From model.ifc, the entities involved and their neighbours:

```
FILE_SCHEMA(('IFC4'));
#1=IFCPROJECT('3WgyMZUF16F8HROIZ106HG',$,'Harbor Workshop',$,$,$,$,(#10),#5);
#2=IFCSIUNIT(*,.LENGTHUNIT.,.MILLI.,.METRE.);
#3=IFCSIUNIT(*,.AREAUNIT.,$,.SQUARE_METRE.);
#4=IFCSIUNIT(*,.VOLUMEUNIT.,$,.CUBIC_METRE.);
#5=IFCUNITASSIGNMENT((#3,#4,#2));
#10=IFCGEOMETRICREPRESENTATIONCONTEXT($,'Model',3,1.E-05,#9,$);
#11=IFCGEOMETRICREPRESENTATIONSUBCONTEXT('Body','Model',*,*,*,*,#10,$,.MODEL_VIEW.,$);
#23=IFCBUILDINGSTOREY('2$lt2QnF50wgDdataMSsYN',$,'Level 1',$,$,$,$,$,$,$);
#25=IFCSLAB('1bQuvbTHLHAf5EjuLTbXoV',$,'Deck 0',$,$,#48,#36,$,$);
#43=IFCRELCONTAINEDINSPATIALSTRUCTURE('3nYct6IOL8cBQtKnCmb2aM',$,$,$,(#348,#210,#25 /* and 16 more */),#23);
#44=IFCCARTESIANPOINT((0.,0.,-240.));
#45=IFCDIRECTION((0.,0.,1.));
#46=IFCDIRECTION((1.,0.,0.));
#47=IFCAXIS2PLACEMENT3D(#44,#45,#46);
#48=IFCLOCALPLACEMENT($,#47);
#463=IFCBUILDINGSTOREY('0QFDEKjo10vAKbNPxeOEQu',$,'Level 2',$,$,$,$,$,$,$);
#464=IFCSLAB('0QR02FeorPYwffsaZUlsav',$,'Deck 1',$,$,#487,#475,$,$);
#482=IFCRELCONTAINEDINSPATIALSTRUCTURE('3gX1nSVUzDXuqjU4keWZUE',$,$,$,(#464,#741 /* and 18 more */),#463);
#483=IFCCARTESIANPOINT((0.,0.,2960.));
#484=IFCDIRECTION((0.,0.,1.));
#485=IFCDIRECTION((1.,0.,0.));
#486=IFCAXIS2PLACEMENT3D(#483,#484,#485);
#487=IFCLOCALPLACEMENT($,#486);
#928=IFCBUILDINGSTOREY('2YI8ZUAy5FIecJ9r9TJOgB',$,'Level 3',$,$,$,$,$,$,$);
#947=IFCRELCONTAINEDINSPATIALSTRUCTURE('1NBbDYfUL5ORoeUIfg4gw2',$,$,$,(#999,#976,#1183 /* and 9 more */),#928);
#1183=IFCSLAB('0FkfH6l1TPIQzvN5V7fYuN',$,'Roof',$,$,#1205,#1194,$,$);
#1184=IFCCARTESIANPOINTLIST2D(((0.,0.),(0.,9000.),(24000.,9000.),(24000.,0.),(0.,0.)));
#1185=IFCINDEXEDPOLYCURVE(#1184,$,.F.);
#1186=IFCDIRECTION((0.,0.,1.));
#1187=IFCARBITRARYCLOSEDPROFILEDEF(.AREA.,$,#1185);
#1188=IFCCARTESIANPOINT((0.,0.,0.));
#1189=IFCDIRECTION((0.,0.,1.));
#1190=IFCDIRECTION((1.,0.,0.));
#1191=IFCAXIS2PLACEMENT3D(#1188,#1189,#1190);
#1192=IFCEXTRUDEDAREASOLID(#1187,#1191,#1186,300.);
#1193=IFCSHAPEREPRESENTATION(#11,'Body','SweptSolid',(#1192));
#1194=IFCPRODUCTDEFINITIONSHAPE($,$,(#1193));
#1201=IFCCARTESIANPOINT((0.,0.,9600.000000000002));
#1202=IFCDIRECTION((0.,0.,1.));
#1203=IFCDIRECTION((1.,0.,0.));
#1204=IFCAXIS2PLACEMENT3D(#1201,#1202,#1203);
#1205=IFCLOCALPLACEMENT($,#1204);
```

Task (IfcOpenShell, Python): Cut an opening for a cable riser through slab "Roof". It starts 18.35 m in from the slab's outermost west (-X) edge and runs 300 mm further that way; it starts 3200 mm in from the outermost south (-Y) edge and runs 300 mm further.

```python
import numpy as np
import ifcopenshell
import ifcopenshell.api.feature
import ifcopenshell.api.geometry
import ifcopenshell.api.root
import ifcopenshell.geom
import ifcopenshell.util.placement
import ifcopenshell.util.representation
import ifcopenshell.util.shape
import ifcopenshell.util.unit

model = ifcopenshell.open("model.ifc")
unit_scale = ifcopenshell.util.unit.calculate_unit_scale(model)
settings = ifcopenshell.geom.settings()


def volume(element):
    """Net volume in cubic metres, openings subtracted."""
    shape = ifcopenshell.geom.create_shape(settings, element)
    return ifcopenshell.util.shape.get_volume(shape.geometry)


slab = model.by_id(1183)
before = volume(slab)

# Extent in the slab's own axes, in metres. The edges named are its -X and -Y sides.
slab_shape = ifcopenshell.geom.create_shape(settings, slab)
vertices = ifcopenshell.util.shape.get_vertices(slab_shape.geometry)
x_min, y_min, bottom = vertices.min(axis=0)
top = vertices[:, 2].max()

opening = ifcopenshell.api.root.create_entity(model, ifc_class="IfcOpeningElement", name="Cable riser opening", predefined_type="OPENING")
context = ifcopenshell.util.representation.get_context(model, "Model", "Body", "MODEL_VIEW")
width, depth = 0.3, 0.3
outline = [(0.0, 0.0), (width, 0.0), (width, depth), (0.0, depth), (0.0, 0.0)]
# Overshoot both faces by 50 mm so the cut is clean.
shape = ifcopenshell.api.geometry.add_slab_representation(
    model, context=context, depth=top - bottom + 0.1, polyline=outline
)
ifcopenshell.api.geometry.assign_representation(model, product=opening, representation=shape)

matrix = ifcopenshell.util.placement.get_local_placement(slab.ObjectPlacement)
matrix[:, 3] = matrix @ np.append(np.array([x_min + 18.35, y_min + 3.2, bottom - 0.05]) / unit_scale, 1.0)
ifcopenshell.api.geometry.edit_object_placement(model, product=opening, matrix=matrix, is_si=False)
ifcopenshell.api.feature.add_feature(model, feature=opening, element=slab)

after = volume(slab)

print(f"slab volume {before:.3f} -> {after:.3f} m3")

model.write("model_v2.ifc")
```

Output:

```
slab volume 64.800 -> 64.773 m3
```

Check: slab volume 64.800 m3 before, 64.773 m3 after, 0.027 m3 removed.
